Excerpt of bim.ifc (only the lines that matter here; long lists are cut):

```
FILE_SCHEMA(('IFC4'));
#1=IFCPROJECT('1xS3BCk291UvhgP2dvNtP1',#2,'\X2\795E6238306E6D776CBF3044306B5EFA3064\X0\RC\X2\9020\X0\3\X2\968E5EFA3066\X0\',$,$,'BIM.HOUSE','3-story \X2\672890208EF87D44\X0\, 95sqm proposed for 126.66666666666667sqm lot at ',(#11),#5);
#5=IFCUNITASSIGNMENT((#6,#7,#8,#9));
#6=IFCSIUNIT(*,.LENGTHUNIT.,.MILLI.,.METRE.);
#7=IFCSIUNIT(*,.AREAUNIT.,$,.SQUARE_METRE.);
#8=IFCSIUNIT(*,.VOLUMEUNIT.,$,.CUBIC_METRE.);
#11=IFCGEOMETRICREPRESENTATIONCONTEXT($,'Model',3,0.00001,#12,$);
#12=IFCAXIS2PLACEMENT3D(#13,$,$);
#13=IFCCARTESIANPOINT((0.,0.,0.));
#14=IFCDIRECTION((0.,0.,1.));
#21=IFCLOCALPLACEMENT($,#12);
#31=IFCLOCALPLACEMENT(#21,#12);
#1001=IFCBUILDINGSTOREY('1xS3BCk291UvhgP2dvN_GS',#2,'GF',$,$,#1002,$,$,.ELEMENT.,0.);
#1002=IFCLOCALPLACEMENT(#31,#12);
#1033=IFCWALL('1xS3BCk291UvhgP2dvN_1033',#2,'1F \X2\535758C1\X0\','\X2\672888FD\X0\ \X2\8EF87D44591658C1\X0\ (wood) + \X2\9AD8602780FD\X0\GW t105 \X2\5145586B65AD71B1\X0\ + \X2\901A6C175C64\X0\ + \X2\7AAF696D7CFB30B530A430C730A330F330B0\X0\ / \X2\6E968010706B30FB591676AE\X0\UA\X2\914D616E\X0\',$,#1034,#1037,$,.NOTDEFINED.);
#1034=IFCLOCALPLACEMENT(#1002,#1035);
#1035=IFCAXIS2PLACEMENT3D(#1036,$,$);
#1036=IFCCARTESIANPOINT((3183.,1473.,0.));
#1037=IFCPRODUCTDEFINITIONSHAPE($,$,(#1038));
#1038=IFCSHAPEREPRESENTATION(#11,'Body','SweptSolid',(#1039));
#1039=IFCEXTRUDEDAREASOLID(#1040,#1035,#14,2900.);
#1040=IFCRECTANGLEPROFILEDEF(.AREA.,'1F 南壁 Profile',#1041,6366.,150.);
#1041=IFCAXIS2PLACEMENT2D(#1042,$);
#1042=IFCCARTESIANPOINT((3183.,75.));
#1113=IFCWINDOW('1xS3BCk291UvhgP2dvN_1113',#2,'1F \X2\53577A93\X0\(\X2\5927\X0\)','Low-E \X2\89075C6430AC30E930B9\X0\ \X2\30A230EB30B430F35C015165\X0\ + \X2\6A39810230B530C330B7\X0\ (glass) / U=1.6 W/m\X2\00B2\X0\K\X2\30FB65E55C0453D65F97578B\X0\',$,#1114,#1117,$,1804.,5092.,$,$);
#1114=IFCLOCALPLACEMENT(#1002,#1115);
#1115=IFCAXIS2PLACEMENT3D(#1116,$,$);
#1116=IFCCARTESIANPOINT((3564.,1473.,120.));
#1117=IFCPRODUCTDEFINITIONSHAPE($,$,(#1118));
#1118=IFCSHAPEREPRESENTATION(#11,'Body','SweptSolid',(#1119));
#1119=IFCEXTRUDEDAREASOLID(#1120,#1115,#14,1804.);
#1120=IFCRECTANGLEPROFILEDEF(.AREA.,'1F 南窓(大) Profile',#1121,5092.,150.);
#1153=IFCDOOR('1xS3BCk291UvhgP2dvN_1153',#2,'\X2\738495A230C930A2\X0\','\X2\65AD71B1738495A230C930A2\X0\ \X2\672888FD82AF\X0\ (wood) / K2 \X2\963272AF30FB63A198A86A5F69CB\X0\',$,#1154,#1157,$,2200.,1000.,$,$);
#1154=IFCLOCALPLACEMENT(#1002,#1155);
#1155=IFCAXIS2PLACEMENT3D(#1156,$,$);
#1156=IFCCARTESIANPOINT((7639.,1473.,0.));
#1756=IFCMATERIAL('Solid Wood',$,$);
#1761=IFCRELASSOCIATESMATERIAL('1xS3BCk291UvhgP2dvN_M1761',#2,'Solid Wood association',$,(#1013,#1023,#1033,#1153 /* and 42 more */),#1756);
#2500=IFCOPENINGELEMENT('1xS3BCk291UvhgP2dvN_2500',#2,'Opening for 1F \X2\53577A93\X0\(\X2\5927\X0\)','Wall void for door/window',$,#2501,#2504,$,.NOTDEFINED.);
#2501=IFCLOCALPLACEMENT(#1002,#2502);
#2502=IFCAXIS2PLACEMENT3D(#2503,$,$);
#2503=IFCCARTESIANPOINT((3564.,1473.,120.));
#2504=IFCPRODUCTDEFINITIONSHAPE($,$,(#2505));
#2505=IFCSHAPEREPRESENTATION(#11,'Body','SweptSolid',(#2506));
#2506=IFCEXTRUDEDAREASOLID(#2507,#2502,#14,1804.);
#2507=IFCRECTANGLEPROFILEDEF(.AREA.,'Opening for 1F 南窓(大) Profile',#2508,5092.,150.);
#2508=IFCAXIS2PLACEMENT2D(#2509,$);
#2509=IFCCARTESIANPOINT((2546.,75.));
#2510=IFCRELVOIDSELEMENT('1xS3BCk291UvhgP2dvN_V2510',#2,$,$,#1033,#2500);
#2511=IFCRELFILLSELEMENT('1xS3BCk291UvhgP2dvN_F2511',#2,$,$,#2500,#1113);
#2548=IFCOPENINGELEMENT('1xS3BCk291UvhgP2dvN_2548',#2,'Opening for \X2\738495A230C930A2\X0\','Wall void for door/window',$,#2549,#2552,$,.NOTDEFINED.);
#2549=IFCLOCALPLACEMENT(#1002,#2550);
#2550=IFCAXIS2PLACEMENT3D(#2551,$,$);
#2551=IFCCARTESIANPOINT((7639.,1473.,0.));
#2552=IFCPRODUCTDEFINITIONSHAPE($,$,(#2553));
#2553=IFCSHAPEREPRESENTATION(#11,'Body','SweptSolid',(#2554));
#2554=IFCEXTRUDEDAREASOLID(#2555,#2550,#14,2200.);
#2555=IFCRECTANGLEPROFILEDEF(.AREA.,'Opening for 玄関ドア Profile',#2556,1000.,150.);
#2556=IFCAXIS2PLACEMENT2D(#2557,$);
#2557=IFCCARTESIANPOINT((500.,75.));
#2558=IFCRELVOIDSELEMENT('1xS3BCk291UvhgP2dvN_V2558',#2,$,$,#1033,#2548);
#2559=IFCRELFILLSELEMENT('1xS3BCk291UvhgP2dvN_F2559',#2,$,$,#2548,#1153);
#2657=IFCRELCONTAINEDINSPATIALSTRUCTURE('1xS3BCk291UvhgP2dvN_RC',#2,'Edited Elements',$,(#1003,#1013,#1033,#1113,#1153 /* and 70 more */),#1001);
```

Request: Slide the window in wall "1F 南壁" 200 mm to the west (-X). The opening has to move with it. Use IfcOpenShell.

```python
import ifcopenshell
import ifcopenshell.api.geometry
import ifcopenshell.util.placement
import ifcopenshell.util.unit

model = ifcopenshell.open("bim.ifc")
unit_scale = ifcopenshell.util.unit.calculate_unit_scale(model)

window = model.by_guid("1xS3BCk291UvhgP2dvN_1113")
opening = window.FillsVoids[0].RelatingOpeningElement
wall = opening.VoidsElements[0].RelatingBuildingElement

wall_matrix = ifcopenshell.util.placement.get_local_placement(wall.ObjectPlacement)
shift = wall_matrix[:3, 0] * -0.2 / unit_scale
before = ifcopenshell.util.placement.get_local_placement(window.ObjectPlacement)[:3, 3].copy()

# The window is not placed relative to its opening, so move both.
for product in (opening, window):
    matrix = ifcopenshell.util.placement.get_local_placement(product.ObjectPlacement)
    matrix[:3, 3] += shift
    ifcopenshell.api.geometry.edit_object_placement(model, product=product, matrix=matrix, is_si=False)

after = ifcopenshell.util.placement.get_local_placement(window.ObjectPlacement)[:3, 3]
print("window moved by", (after - before).round(3) + 0.0)

model.write("bim_edited.ifc")
```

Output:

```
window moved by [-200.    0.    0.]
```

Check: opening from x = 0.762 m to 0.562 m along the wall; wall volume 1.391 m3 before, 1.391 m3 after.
